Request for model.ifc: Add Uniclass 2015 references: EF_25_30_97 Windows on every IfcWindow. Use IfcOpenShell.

First a look at what the model holds.

```python
import ifcopenshell

model = ifcopenshell.open("model.ifc")
print(model.schema)
print("classifications:", [c.Name for c in model.by_type("IfcClassification")])
for ifc_class in ("IfcDoor", "IfcRoof", "IfcStair", "IfcWall", "IfcWindow"):
    print(ifc_class, len(model.by_type(ifc_class)))
```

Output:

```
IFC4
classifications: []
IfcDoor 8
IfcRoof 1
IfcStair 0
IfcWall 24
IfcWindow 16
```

```python
import ifcopenshell
import ifcopenshell.api.classification

model = ifcopenshell.open("model.ifc")

system = ifcopenshell.api.classification.add_classification(model, classification="Uniclass 2015")

codes = {
    "IfcWindow": ("EF_25_30_97", "Windows"),
}
for ifc_class, (code, name) in codes.items():
    products = model.by_type(ifc_class)
    ifcopenshell.api.classification.add_reference(
        model, products=products, classification=system, identification=code, name=name
    )
    print(code, len(products))

model.write("model_v2.ifc")
```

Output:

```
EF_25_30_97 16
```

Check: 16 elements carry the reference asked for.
